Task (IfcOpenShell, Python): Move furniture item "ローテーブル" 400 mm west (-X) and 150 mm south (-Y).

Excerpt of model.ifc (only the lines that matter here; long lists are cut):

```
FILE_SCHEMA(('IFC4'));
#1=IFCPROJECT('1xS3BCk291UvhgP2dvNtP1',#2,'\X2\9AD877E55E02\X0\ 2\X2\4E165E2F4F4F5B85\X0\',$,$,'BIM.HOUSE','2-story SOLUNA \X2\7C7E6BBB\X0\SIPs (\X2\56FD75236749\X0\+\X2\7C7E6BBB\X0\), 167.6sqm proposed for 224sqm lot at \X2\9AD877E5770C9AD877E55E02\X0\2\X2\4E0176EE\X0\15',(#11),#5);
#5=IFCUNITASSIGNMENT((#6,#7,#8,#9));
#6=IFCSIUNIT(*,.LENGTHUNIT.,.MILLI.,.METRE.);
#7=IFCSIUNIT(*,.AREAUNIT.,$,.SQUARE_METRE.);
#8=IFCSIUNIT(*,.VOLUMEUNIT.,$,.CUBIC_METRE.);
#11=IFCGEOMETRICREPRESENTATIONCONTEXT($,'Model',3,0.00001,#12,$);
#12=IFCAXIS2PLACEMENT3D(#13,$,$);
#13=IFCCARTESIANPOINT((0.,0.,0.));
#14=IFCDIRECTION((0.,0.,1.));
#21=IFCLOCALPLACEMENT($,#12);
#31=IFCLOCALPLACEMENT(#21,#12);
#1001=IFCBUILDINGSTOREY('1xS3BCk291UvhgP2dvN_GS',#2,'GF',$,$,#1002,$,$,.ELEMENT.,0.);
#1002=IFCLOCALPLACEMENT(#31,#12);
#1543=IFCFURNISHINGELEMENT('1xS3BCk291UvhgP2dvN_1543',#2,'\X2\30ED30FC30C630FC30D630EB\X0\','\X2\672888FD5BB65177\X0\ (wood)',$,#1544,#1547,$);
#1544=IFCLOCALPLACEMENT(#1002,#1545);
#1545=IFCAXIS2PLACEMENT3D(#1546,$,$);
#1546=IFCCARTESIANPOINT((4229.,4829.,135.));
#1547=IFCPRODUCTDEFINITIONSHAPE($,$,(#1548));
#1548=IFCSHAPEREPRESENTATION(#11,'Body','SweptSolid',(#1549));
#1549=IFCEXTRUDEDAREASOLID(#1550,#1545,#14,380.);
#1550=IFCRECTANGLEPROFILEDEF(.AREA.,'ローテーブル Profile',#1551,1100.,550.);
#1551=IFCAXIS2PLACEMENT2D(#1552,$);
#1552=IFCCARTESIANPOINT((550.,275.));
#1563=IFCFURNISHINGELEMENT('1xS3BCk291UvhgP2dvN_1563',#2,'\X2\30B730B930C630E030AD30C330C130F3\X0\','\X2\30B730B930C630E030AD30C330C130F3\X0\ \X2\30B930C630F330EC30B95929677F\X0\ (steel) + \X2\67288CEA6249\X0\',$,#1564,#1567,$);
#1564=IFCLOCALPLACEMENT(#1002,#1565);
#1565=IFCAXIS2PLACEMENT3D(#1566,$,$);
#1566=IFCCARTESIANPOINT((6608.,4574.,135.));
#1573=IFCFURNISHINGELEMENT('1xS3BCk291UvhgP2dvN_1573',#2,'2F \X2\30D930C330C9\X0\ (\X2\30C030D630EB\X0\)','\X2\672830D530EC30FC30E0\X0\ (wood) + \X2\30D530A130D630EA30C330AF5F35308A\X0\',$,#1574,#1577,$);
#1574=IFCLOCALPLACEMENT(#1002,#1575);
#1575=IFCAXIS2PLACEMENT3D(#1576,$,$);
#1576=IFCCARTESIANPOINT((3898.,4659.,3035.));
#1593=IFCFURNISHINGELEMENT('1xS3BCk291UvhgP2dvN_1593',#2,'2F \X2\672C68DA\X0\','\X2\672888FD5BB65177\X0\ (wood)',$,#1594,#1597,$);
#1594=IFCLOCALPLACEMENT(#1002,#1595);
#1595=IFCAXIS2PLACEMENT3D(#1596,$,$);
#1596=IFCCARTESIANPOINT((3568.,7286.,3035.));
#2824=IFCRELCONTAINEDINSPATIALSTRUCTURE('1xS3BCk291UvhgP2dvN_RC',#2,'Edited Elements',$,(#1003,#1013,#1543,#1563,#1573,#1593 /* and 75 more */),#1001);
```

```python
import ifcopenshell
import ifcopenshell.api.geometry
import ifcopenshell.util.placement
import ifcopenshell.util.unit

model = ifcopenshell.open("model.ifc")
unit_scale = ifcopenshell.util.unit.calculate_unit_scale(model)

item = model.by_guid("1xS3BCk291UvhgP2dvN_1543")
matrix = ifcopenshell.util.placement.get_local_placement(item.ObjectPlacement)
matrix[0, 3] -= 0.4 / unit_scale
matrix[1, 3] -= 0.15 / unit_scale
ifcopenshell.api.geometry.edit_object_placement(model, product=item, matrix=matrix, is_si=False)

print(ifcopenshell.util.placement.get_local_placement(item.ObjectPlacement).round(3) + 0.0)

model.write("model-out.ifc")
```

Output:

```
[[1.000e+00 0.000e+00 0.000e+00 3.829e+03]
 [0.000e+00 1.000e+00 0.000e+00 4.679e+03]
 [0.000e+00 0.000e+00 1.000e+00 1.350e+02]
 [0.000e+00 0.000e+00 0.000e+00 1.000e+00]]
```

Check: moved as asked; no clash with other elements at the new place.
